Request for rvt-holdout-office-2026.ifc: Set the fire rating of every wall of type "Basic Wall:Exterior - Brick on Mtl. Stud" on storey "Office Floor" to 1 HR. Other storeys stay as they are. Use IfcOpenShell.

First a look at what the model holds.

```python
import ifcopenshell
import ifcopenshell.util.element

model = ifcopenshell.open("rvt-holdout-office-2026.ifc")
print(model.schema)
storey = next(s for s in model.by_type("IfcBuildingStorey") if s.Name == "Office Floor")
walls = [e for e in ifcopenshell.util.element.get_decomposition(storey) if e.is_a("IfcWall")]
seen = {}
for e in walls:
    element_type = ifcopenshell.util.element.get_type(e)
    key = (element_type.Name if element_type != e and element_type else None, ifcopenshell.util.element.get_pset(e, "Pset_WallCommon", "FireRating"))
    seen[key] = seen.get(key, 0) + 1
for (name, value), count in sorted(seen.items(), key=str):
    print(count, "x", name, "|", value)
```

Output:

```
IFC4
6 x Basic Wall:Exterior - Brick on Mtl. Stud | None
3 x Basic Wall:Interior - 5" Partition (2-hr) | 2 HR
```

```python
import ifcopenshell
import ifcopenshell.api.pset
import ifcopenshell.util.element

model = ifcopenshell.open("rvt-holdout-office-2026.ifc")

storey = next(s for s in model.by_type("IfcBuildingStorey") if s.Name == "Office Floor")
walls = [e for e in ifcopenshell.util.element.get_decomposition(storey) if e.is_a("IfcWall")]

count = 0
for e in walls:
    element_type = ifcopenshell.util.element.get_type(e)
    if element_type in (None, e) or element_type.Name != "Basic Wall:Exterior - Brick on Mtl. Stud":
        continue
    # add_pset returns the element's existing set when there is one.
    pset = ifcopenshell.api.pset.add_pset(model, product=e, name="Pset_WallCommon")
    ifcopenshell.api.pset.edit_pset(model, pset=pset, properties={"FireRating": "1 HR"})
    count += 1

print(count, "walls updated")

model.write("rvt-holdout-office-2026-out.ifc")
```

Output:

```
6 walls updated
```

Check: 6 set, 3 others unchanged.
